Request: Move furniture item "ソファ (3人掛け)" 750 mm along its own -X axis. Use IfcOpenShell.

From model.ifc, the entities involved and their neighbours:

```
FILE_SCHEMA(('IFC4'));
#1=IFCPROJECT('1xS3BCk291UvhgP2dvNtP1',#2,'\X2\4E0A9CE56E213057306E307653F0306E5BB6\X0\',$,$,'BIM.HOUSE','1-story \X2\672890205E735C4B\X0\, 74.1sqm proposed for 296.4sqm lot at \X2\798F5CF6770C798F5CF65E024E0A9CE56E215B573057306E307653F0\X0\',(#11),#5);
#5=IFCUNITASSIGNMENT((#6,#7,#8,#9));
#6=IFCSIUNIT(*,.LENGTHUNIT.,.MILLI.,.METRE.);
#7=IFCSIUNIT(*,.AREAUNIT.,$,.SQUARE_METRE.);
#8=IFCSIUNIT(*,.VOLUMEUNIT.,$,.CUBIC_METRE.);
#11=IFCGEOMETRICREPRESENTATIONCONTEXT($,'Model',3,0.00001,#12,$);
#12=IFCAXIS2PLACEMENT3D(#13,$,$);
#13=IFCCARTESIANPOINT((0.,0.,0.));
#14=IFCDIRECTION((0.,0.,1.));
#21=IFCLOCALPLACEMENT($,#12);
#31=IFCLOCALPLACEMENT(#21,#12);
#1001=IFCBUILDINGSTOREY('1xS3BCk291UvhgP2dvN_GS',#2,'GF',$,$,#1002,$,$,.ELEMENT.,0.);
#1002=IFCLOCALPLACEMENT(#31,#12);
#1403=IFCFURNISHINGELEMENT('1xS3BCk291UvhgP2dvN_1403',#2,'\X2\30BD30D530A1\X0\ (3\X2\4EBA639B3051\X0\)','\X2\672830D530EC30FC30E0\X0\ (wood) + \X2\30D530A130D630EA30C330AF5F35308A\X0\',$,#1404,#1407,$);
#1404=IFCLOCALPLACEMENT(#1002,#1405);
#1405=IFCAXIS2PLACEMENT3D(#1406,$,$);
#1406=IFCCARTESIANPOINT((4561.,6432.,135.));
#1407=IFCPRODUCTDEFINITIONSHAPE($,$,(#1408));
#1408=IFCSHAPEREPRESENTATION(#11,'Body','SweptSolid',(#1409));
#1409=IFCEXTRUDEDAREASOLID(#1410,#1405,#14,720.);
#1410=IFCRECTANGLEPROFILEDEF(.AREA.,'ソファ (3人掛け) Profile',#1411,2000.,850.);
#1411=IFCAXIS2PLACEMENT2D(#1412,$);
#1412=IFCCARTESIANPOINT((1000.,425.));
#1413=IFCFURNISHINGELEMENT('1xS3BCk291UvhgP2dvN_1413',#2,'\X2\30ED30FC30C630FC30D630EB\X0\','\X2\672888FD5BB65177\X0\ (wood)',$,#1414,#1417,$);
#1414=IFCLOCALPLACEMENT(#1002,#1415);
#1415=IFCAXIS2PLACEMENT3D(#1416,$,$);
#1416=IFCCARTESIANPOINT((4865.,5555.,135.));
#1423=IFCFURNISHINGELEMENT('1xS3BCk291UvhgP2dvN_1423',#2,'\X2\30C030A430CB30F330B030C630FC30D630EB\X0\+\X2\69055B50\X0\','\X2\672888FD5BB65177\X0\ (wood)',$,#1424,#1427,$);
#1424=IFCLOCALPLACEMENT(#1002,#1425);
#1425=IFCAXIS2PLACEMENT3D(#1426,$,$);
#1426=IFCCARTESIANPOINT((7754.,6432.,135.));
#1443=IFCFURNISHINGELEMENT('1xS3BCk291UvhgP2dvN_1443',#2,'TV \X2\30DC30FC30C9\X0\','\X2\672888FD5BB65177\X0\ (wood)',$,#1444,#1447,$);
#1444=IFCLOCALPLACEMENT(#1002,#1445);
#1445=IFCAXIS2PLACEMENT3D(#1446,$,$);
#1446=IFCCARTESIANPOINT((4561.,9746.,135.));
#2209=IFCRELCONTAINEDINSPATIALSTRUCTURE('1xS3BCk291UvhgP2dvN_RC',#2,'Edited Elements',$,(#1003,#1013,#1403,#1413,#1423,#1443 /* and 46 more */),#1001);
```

```python
import ifcopenshell
import ifcopenshell.api.geometry
import ifcopenshell.util.placement

model = ifcopenshell.open("model.ifc")

item = model.by_guid("1xS3BCk291UvhgP2dvN_1403")
matrix = ifcopenshell.util.placement.get_local_placement(item.ObjectPlacement)
matrix[:3, 3] -= matrix[:3, 0] * 750.0
ifcopenshell.api.geometry.edit_object_placement(model, product=item, matrix=matrix, is_si=False)

print(ifcopenshell.util.placement.get_local_placement(item.ObjectPlacement).round(3) + 0.0)

model.write("model_edited.ifc")
```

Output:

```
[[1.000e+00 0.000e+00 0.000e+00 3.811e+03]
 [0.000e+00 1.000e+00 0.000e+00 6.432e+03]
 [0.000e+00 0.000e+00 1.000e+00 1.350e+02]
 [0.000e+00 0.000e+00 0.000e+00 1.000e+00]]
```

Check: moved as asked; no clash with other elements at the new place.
